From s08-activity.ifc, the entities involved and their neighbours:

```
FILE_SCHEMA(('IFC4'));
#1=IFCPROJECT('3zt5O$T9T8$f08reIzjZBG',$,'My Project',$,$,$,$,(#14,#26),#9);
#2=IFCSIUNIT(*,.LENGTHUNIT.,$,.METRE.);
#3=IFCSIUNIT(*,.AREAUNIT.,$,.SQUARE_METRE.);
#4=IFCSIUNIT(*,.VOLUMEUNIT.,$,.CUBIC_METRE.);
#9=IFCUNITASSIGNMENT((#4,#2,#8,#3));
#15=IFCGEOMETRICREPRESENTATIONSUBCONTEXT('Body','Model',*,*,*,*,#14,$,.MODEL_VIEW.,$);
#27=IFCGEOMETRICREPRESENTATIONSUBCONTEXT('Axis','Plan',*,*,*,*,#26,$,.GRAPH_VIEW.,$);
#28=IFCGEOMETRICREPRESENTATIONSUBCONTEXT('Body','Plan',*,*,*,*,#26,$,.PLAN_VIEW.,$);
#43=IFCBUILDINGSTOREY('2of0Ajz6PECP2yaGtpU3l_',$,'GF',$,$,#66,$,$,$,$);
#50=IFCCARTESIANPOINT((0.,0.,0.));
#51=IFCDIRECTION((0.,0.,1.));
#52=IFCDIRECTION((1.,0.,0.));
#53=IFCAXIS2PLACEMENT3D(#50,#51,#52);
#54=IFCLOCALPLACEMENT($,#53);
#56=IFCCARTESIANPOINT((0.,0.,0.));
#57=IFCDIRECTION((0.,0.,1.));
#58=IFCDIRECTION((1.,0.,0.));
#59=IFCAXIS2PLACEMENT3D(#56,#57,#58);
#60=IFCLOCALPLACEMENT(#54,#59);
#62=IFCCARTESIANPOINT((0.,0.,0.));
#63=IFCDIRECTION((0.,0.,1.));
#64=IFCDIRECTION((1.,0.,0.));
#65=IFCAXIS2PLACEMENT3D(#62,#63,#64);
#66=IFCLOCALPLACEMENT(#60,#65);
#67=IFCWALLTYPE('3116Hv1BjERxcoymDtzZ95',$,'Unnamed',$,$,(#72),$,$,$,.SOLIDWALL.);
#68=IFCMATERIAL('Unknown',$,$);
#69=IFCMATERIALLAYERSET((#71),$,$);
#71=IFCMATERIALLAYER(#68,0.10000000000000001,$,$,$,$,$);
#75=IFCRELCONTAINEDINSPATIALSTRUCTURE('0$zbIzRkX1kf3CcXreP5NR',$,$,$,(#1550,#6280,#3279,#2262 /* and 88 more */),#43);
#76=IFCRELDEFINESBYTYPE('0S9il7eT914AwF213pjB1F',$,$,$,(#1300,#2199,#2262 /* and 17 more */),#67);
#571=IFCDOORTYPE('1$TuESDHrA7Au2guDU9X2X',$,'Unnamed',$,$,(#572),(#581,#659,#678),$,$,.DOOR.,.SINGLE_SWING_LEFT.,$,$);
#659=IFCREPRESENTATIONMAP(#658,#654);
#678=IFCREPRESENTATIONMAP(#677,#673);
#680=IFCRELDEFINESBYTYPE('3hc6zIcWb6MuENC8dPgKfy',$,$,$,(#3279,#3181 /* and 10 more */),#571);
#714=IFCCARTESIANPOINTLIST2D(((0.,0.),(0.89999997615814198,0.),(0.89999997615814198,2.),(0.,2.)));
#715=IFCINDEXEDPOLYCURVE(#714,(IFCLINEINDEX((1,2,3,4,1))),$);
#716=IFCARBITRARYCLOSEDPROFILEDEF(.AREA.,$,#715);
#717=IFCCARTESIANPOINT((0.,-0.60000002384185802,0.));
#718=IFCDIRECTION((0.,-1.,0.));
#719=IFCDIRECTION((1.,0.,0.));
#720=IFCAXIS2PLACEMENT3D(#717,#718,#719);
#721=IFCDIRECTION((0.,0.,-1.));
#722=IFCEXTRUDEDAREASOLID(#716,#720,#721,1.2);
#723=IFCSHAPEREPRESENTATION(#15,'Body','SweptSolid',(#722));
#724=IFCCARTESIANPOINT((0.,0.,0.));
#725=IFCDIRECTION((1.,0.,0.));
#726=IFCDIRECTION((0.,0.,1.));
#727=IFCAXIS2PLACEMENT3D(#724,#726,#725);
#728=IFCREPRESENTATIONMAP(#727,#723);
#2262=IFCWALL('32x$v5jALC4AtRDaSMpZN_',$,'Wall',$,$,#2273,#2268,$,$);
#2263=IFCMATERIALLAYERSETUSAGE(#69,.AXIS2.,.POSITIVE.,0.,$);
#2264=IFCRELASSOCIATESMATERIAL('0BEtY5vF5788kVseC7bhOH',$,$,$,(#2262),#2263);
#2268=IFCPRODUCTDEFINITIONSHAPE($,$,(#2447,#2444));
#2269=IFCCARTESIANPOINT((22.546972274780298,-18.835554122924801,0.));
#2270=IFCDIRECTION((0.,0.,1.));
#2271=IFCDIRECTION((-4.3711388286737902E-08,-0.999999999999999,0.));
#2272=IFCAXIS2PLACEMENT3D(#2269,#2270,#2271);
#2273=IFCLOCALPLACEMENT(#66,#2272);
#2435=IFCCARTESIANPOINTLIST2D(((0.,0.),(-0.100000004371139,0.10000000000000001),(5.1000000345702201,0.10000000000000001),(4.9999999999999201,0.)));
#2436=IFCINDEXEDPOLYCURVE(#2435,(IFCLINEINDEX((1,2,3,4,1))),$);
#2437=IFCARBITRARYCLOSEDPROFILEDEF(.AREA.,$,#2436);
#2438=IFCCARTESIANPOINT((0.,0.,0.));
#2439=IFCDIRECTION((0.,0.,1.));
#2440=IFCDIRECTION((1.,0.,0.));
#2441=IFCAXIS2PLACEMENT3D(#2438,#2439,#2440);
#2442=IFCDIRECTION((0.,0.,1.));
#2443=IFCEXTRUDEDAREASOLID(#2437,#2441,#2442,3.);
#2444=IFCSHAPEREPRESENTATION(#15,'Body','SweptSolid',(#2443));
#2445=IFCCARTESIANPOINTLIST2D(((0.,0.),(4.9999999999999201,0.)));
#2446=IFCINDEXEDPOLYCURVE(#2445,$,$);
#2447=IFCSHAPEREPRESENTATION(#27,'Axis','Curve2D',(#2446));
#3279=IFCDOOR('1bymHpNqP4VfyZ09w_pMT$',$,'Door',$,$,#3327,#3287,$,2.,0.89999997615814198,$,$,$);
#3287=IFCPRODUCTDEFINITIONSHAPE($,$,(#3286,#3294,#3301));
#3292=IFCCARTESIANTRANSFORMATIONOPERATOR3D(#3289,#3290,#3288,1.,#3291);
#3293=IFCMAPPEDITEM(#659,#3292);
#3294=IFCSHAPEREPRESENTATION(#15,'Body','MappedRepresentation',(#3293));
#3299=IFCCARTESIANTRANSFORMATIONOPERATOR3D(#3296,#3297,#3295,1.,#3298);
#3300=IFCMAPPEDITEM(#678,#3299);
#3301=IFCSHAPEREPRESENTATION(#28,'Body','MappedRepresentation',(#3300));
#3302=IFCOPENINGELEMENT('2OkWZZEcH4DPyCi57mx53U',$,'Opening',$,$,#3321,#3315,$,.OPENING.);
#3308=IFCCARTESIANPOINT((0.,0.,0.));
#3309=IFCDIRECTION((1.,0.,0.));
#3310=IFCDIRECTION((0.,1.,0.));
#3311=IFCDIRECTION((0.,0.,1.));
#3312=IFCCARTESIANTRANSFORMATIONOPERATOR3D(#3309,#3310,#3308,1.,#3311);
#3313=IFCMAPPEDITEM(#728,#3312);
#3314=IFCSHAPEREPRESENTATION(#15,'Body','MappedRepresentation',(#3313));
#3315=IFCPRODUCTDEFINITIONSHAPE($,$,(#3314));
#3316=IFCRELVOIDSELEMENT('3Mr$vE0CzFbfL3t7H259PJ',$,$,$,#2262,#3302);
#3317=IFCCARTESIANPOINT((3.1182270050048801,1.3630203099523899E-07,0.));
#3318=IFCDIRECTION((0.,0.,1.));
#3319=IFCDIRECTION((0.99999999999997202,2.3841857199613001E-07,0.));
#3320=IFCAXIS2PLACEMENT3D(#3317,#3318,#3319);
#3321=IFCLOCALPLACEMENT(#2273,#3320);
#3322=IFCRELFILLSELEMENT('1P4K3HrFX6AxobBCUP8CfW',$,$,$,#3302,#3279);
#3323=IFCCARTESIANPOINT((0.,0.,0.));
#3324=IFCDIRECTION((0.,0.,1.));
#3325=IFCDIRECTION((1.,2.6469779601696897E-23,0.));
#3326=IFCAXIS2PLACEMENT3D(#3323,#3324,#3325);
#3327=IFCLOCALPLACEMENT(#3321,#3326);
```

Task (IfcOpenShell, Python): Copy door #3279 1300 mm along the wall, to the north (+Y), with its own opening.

```python
import ifcopenshell
import ifcopenshell.api.feature
import ifcopenshell.api.geometry
import ifcopenshell.api.root
import ifcopenshell.geom
import ifcopenshell.util.element
import ifcopenshell.util.placement
import ifcopenshell.util.shape
import ifcopenshell.util.unit

model = ifcopenshell.open("s08-activity.ifc")
unit_scale = ifcopenshell.util.unit.calculate_unit_scale(model)
settings = ifcopenshell.geom.settings()


def volume(element):
    """Net volume in cubic metres, openings subtracted."""
    shape = ifcopenshell.geom.create_shape(settings, element)
    return ifcopenshell.util.shape.get_volume(shape.geometry)


door = model.by_guid("1bymHpNqP4VfyZ09w_pMT$")
opening = door.FillsVoids[0].RelatingOpeningElement
wall = opening.VoidsElements[0].RelatingBuildingElement
before = volume(wall)
shift = ifcopenshell.util.placement.get_local_placement(wall.ObjectPlacement)[:3, 0] * -1.3 / unit_scale

# copy_class copies the void relationship, type, container and properties, but no geometry.
new_opening = ifcopenshell.api.root.copy_class(model, product=opening)
new_opening.Representation = ifcopenshell.util.element.copy_deep(
    model, opening.Representation, exclude=["IfcGeometricRepresentationContext", "IfcRepresentationMap"]
)
new_door = ifcopenshell.api.root.copy_class(model, product=door)
new_door.Representation = ifcopenshell.util.element.copy_deep(
    model, door.Representation, exclude=["IfcGeometricRepresentationContext", "IfcRepresentationMap"]
)
ifcopenshell.api.feature.add_filling(model, opening=new_opening, element=new_door)

for old, new in ((opening, new_opening), (door, new_door)):
    matrix = ifcopenshell.util.placement.get_local_placement(old.ObjectPlacement)
    matrix[:3, 3] += shift
    ifcopenshell.api.geometry.edit_object_placement(model, product=new, matrix=matrix, is_si=False)

after = volume(wall)

print(f"wall volume {before:.3f} -> {after:.3f} m3")

model.write("s08-activity-out.ifc")
```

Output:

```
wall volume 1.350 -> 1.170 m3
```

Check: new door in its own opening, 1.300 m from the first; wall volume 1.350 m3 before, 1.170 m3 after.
